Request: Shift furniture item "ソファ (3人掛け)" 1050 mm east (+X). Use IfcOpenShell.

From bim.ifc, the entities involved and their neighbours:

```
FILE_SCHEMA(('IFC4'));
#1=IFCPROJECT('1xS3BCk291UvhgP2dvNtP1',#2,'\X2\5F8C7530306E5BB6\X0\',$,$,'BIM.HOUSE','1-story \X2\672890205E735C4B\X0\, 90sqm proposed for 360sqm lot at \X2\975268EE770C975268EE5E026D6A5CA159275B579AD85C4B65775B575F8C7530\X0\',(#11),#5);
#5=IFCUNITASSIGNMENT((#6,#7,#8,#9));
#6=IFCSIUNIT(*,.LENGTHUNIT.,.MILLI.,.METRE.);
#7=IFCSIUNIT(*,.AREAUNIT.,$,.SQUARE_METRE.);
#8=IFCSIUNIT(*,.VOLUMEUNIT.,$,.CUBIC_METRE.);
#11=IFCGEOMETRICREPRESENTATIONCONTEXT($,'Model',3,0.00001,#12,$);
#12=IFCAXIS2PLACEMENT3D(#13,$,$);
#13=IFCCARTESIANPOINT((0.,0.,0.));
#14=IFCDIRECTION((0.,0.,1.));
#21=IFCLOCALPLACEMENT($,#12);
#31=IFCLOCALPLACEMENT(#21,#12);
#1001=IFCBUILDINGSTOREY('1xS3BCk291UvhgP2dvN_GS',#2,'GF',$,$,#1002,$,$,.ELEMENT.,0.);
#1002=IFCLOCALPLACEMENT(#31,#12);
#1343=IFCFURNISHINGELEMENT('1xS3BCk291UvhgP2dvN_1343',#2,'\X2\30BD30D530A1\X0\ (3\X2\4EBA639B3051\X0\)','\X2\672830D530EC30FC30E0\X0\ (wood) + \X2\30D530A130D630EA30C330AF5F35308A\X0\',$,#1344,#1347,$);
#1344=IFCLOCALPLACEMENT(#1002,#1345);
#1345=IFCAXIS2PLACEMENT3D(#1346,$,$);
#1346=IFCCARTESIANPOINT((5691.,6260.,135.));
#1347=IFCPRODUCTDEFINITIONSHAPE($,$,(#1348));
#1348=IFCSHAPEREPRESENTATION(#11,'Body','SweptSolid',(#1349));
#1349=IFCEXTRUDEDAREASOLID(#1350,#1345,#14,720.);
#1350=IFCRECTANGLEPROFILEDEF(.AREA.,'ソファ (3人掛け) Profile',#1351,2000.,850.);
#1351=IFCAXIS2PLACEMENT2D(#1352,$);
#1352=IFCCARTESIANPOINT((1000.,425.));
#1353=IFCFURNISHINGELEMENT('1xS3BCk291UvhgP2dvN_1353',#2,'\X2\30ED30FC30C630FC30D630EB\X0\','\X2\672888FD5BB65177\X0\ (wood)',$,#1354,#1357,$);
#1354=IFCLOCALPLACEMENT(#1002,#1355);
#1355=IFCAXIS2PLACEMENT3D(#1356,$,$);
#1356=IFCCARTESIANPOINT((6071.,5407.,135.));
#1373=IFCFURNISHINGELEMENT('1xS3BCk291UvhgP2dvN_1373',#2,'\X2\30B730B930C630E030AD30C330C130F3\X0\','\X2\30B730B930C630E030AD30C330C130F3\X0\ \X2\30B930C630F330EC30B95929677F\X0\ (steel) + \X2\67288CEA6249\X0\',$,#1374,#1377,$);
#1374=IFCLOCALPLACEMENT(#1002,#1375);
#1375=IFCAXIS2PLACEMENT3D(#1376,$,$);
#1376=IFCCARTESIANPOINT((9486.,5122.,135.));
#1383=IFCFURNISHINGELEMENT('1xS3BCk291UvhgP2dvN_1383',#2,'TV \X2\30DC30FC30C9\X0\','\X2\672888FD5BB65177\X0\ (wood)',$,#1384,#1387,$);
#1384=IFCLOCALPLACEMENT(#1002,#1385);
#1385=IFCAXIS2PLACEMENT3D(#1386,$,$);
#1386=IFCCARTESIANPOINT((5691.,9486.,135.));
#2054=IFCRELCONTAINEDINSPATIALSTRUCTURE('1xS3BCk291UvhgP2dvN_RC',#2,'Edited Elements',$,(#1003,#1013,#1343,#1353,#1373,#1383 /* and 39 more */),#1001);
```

```python
import ifcopenshell
import ifcopenshell.api.geometry
import ifcopenshell.util.placement
import ifcopenshell.util.unit

model = ifcopenshell.open("bim.ifc")
unit_scale = ifcopenshell.util.unit.calculate_unit_scale(model)

item = model.by_guid("1xS3BCk291UvhgP2dvN_1343")
matrix = ifcopenshell.util.placement.get_local_placement(item.ObjectPlacement)
matrix[0, 3] += 1.05 / unit_scale
ifcopenshell.api.geometry.edit_object_placement(model, product=item, matrix=matrix, is_si=False)

print(ifcopenshell.util.placement.get_local_placement(item.ObjectPlacement).round(3) + 0.0)

model.write("bim_v2.ifc")
```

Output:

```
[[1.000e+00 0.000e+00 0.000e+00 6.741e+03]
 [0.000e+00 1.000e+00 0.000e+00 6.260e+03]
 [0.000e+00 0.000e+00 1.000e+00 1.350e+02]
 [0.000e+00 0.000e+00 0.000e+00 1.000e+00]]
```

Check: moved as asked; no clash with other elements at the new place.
